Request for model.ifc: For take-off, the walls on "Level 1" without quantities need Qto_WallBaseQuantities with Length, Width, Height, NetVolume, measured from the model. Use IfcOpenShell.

First a look at what the model holds.

```python
import ifcopenshell
import ifcopenshell.util.element
import ifcopenshell.util.unit

model = ifcopenshell.open("model.ifc")
print(model.schema)
for unit_type in ("LENGTHUNIT", "AREAUNIT", "VOLUMEUNIT"):
    print(unit_type, ifcopenshell.util.unit.calculate_unit_scale(model, unit_type))
storey = next(s for s in model.by_type("IfcBuildingStorey") if s.Name == "Level 1")
walls = [e for e in ifcopenshell.util.element.get_decomposition(storey) if e.is_a("IfcWall")]
for e in sorted(walls, key=lambda e: e.id()):
    print(e.id(), e.is_a(), e.Name, list(ifcopenshell.util.element.get_psets(e, qtos_only=True)), sep=" | ")
```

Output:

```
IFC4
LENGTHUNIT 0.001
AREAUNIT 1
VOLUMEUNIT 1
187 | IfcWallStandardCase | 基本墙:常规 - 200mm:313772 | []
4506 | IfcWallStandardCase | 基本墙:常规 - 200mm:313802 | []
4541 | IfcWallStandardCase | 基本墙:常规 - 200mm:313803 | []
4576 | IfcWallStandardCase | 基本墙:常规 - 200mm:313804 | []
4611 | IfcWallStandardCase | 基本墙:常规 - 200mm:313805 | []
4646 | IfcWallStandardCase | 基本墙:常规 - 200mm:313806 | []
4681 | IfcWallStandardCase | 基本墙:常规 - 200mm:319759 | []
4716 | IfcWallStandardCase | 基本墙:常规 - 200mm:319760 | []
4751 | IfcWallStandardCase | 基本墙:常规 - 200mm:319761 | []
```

```python
import ifcopenshell
import ifcopenshell.api.pset
import ifcopenshell.geom
import ifcopenshell.util.element
import ifcopenshell.util.shape
import ifcopenshell.util.unit

model = ifcopenshell.open("model.ifc")
unit_scale = ifcopenshell.util.unit.calculate_unit_scale(model)
volume_scale = ifcopenshell.util.unit.calculate_unit_scale(model, "VOLUMEUNIT")
settings = ifcopenshell.geom.settings()

storey = next(s for s in model.by_type("IfcBuildingStorey") if s.Name == "Level 1")
walls = [e for e in ifcopenshell.util.element.get_decomposition(storey) if e.is_a("IfcWall")]

for e in sorted(walls, key=lambda e: e.id()):
    if ifcopenshell.util.element.get_psets(e, qtos_only=True, should_inherit=False):
        continue
    # Geometry comes back in metres, in the element's own axes.
    shape = ifcopenshell.geom.create_shape(settings, e)
    values = {
        "Length": ifcopenshell.util.shape.get_x(shape.geometry) / unit_scale,
        "Width": ifcopenshell.util.shape.get_y(shape.geometry) / unit_scale,
        "Height": ifcopenshell.util.shape.get_z(shape.geometry) / unit_scale,
        "NetVolume": ifcopenshell.util.shape.get_volume(shape.geometry) / volume_scale,
    }
    qto = ifcopenshell.api.pset.add_qto(model, product=e, name="Qto_WallBaseQuantities")
    ifcopenshell.api.pset.edit_qto(model, qto=qto, properties=values)
    print(e.id(), {k: round(v, 3) for k, v in values.items()})

model.write("model_updated.ifc")
```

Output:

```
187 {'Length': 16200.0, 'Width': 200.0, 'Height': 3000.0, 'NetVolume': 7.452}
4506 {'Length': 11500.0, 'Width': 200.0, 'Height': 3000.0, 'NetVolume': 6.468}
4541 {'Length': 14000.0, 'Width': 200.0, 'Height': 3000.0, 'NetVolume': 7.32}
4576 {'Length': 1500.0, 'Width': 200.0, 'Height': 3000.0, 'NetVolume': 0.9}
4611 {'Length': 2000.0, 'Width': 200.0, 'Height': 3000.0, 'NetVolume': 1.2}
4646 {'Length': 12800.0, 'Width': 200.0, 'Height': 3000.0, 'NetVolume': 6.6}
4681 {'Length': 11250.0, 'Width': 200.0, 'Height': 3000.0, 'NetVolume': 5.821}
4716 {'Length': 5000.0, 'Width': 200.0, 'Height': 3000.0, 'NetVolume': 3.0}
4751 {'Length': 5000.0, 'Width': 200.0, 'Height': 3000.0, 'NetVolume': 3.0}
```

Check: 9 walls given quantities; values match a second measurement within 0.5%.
